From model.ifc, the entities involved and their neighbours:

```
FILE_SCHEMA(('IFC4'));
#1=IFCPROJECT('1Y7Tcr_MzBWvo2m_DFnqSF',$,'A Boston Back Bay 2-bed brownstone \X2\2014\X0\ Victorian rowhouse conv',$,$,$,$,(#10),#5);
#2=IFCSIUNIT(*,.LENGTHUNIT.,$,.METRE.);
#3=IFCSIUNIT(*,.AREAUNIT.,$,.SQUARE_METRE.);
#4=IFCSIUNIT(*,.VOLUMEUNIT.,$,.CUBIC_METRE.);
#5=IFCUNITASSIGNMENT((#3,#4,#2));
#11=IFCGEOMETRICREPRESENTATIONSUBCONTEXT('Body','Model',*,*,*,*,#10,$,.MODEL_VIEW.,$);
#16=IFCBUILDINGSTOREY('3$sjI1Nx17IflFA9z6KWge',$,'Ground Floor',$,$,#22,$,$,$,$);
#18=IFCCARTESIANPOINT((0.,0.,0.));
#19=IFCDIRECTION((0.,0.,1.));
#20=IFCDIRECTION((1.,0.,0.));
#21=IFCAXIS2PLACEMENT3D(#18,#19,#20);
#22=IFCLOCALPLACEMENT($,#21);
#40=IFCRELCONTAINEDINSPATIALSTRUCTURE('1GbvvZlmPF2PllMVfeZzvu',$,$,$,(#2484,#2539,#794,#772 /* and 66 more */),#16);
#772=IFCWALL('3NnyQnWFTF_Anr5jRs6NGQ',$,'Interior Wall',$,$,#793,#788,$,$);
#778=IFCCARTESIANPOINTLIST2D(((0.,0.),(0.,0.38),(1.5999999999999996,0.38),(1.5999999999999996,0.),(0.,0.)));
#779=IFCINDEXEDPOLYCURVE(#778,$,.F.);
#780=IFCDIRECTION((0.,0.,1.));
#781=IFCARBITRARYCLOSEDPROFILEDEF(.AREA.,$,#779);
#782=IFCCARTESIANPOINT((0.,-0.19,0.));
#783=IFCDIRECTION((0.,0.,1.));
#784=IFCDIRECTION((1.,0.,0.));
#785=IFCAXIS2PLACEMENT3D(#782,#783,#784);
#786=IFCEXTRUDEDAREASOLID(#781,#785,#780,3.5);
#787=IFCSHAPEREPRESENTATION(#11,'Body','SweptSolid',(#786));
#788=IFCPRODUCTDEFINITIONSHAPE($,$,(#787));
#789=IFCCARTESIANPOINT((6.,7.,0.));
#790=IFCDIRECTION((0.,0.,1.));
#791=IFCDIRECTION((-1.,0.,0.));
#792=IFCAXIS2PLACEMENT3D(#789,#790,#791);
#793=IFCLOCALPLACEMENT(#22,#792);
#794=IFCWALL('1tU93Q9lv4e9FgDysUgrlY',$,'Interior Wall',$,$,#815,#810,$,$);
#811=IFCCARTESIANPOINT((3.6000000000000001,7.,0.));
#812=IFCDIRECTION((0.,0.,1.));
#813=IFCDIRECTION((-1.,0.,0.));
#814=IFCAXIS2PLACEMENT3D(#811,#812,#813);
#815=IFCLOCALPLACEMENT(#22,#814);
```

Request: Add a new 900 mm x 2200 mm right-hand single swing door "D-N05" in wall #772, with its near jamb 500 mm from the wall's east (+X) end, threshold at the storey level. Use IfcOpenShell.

```python
import numpy as np
import ifcopenshell
import ifcopenshell.api.feature
import ifcopenshell.api.geometry
import ifcopenshell.api.root
import ifcopenshell.api.spatial
import ifcopenshell.geom
import ifcopenshell.util.element
import ifcopenshell.util.placement
import ifcopenshell.util.representation
import ifcopenshell.util.shape
import ifcopenshell.util.unit

model = ifcopenshell.open("model.ifc")
unit_scale = ifcopenshell.util.unit.calculate_unit_scale(model)
settings = ifcopenshell.geom.settings()


def volume(element):
    """Net volume in cubic metres, openings subtracted."""
    shape = ifcopenshell.geom.create_shape(settings, element)
    return ifcopenshell.util.shape.get_volume(shape.geometry)


wall = model.by_guid("3NnyQnWFTF_Anr5jRs6NGQ")
storey = ifcopenshell.util.element.get_container(wall, ifc_class="IfcBuildingStorey")
context = ifcopenshell.util.representation.get_context(model, "Model", "Body", "MODEL_VIEW")
before = volume(wall)

width, height, from_end, sill = 0.9, 2.2, 0.5, 0.0  # metres

# The wall runs along its own X axis, and the end named is its -X end.
wall_shape = ifcopenshell.geom.create_shape(settings, wall)
x, y, z = ifcopenshell.util.shape.get_vertices(wall_shape.geometry).T
start = x.min() + from_end
face, thickness = float(y.min()), float(y.max() - y.min())
wall_matrix = ifcopenshell.util.placement.get_local_placement(wall.ObjectPlacement)
level = ifcopenshell.util.placement.get_local_placement(storey.ObjectPlacement)[2, 3]


def in_wall(x, y):
    """Placement at x, y metres in the wall's axes, at sill height."""
    matrix = wall_matrix.copy()
    matrix[:, 3] = wall_matrix @ np.array([x / unit_scale, y / unit_scale, 0.0, 1.0])
    matrix[2, 3] = level + sill / unit_scale
    return matrix


# Opening: a box that overshoots both wall faces by 50 mm.
opening = ifcopenshell.api.root.create_entity(model, ifc_class="IfcOpeningElement", predefined_type="OPENING")
box = ifcopenshell.api.geometry.add_wall_representation(
    model, context=context, length=width, height=height, thickness=thickness + 0.1
)
ifcopenshell.api.geometry.assign_representation(model, product=opening, representation=box)
ifcopenshell.api.geometry.edit_object_placement(model, product=opening, matrix=in_wall(start, face - 0.05), is_si=False)
ifcopenshell.api.feature.add_feature(model, feature=opening, element=wall)

door = ifcopenshell.api.root.create_entity(model, ifc_class="IfcDoor", name="D-N05", predefined_type="DOOR")
door.OverallWidth, door.OverallHeight = width / unit_scale, height / unit_scale
door.OperationType = "SINGLE_SWING_RIGHT"
body = ifcopenshell.api.geometry.add_door_representation(
    model,
    context=context,
    overall_width=door.OverallWidth,
    overall_height=door.OverallHeight,
    operation_type="SINGLE_SWING_RIGHT",
    lining_properties={"LiningDepth": thickness / unit_scale, "ThresholdDepth": thickness / unit_scale},
)
ifcopenshell.api.geometry.assign_representation(model, product=door, representation=body)
ifcopenshell.api.spatial.assign_container(model, products=[door], relating_structure=storey)
ifcopenshell.api.feature.add_filling(model, opening=opening, element=door)

# The lining spans the wall, so the door starts at the wall face.
ifcopenshell.api.geometry.edit_object_placement(model, product=door, matrix=in_wall(start, face), is_si=False)

after = volume(wall)

print(f"wall volume {before:.3f} -> {after:.3f} m3")

model.write("model_edited.ifc")
```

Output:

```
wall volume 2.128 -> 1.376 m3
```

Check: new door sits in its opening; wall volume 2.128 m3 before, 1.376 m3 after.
